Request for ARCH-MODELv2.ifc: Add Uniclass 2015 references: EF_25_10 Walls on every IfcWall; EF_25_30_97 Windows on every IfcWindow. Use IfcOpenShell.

First a look at what the model holds.

```python
import ifcopenshell

model = ifcopenshell.open("ARCH-MODELv2.ifc")
print(model.schema)
print("classifications:", [c.Name for c in model.by_type("IfcClassification")])
for ifc_class in ("IfcDoor", "IfcRoof", "IfcStair", "IfcWall", "IfcWindow"):
    print(ifc_class, len(model.by_type(ifc_class)))
```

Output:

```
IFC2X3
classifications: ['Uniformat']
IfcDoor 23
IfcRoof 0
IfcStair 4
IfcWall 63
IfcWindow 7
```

```python
import ifcopenshell
import ifcopenshell.api.classification

model = ifcopenshell.open("ARCH-MODELv2.ifc")

# IFC2X3 requires Source and Edition and has no link from the project to the system.
system = model.create_entity("IfcClassification", Source="NBS", Edition="2015", Name="Uniclass 2015")

codes = {
    "IfcWall": ("EF_25_10", "Walls"),
    "IfcWindow": ("EF_25_30_97", "Windows"),
}
for ifc_class, (code, name) in codes.items():
    products = model.by_type(ifc_class)
    ifcopenshell.api.classification.add_reference(
        model, products=products, classification=system, identification=code, name=name
    )
    print(code, len(products))

model.write("ARCH-MODELv2_updated.ifc")
```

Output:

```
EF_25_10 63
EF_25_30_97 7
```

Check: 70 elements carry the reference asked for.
